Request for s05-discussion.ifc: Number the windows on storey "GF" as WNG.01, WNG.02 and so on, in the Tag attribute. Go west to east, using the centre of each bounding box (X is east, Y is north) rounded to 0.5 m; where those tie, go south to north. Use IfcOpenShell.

First a look at what the model holds.

```python
import ifcopenshell
import ifcopenshell.util.element
import ifcopenshell.util.placement

model = ifcopenshell.open("s05-discussion.ifc")
print(model.schema)
storey = next(s for s in model.by_type("IfcBuildingStorey") if s.Name == "GF")
windows = [e for e in ifcopenshell.util.element.get_decomposition(storey) if e.is_a("IfcWindow")]
for e in sorted(windows, key=lambda e: e.id()):
    origin = ifcopenshell.util.placement.get_local_placement(e.ObjectPlacement)[:3, 3]
    print(e.id(), e.Tag, e.Name, origin.round(2) + 0.0, sep=" | ")
```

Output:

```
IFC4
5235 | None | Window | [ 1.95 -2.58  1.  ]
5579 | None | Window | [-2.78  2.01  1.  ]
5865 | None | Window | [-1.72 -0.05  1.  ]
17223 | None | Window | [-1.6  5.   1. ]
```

```python
import ifcopenshell
import ifcopenshell.geom
import ifcopenshell.util.element
import ifcopenshell.util.shape

model = ifcopenshell.open("s05-discussion.ifc")
settings = ifcopenshell.geom.settings()
settings.set("use-world-coords", True)


def centre(element):
    shape = ifcopenshell.geom.create_shape(settings, element)
    return ifcopenshell.util.shape.get_bbox_centroid(shape.geometry)


storey = next(s for s in model.by_type("IfcBuildingStorey") if s.Name == "GF")
windows = [e for e in ifcopenshell.util.element.get_decomposition(storey) if e.is_a("IfcWindow")]

# Insertion points can sit at a corner or the storey origin, so sort by the geometry (in metres).
centres = {e: centre(e) for e in windows}
windows.sort(key=lambda e: (round(centres[e][0] / 0.5), centres[e][1]))

for i, e in enumerate(windows, start=1):
    number = f"WNG.{i:02d}"
    e.Tag = number
    print(e.id(), number)

model.write("s05-discussion_updated.ifc")
```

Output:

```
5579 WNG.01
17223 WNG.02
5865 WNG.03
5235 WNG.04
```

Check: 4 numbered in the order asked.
